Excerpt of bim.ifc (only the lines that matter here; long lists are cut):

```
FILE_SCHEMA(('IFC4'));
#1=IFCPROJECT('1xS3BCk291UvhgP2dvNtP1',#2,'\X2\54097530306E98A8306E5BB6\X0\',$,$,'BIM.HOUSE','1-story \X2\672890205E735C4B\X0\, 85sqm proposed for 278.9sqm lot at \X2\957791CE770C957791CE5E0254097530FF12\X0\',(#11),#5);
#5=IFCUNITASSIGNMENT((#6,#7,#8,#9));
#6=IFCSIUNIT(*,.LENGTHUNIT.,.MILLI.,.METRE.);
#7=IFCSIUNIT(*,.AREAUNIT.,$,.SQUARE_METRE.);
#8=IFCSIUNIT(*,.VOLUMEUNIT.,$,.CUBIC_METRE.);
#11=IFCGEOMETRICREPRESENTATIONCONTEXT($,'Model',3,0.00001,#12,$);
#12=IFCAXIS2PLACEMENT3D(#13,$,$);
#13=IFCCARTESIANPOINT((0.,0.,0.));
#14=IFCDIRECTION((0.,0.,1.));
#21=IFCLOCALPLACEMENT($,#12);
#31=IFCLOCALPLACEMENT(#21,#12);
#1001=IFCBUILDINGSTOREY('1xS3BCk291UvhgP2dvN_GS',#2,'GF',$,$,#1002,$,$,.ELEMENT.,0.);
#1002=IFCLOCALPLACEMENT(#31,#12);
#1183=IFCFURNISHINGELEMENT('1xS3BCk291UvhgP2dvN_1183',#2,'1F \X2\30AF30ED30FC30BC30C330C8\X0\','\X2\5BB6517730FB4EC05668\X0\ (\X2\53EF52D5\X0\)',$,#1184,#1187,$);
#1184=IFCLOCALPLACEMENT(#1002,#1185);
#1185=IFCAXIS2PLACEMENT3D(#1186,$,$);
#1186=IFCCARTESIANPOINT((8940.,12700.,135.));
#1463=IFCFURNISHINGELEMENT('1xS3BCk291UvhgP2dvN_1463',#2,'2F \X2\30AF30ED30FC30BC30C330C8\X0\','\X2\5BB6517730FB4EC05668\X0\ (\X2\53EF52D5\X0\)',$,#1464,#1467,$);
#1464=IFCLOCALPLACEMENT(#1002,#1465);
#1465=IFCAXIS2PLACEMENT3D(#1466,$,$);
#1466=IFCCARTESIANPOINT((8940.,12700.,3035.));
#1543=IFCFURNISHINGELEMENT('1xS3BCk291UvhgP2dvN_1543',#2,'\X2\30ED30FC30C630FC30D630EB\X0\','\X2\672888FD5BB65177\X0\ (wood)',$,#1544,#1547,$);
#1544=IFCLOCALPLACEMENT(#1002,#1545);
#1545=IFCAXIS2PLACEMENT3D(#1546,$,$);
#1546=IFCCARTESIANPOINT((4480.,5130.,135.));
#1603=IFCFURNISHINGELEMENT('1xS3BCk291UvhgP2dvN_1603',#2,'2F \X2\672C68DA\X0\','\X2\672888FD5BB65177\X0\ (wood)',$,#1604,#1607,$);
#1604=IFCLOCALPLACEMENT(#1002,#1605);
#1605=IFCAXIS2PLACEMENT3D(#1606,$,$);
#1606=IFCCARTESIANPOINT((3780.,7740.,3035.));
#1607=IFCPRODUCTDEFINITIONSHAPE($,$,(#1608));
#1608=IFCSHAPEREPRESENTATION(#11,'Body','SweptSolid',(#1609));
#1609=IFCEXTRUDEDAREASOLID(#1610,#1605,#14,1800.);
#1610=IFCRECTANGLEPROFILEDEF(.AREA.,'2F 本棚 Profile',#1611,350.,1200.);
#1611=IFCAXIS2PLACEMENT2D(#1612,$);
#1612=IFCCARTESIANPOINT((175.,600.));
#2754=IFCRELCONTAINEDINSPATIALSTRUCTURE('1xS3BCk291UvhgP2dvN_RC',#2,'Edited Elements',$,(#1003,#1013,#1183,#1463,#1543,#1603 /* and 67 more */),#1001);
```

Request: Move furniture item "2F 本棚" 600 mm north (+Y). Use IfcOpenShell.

```python
import ifcopenshell
import ifcopenshell.api.geometry
import ifcopenshell.util.placement
import ifcopenshell.util.unit

model = ifcopenshell.open("bim.ifc")
unit_scale = ifcopenshell.util.unit.calculate_unit_scale(model)

item = model.by_guid("1xS3BCk291UvhgP2dvN_1603")
matrix = ifcopenshell.util.placement.get_local_placement(item.ObjectPlacement)
matrix[1, 3] += 0.6 / unit_scale
ifcopenshell.api.geometry.edit_object_placement(model, product=item, matrix=matrix, is_si=False)

print(ifcopenshell.util.placement.get_local_placement(item.ObjectPlacement).round(3) + 0.0)

model.write("bim_edited.ifc")
```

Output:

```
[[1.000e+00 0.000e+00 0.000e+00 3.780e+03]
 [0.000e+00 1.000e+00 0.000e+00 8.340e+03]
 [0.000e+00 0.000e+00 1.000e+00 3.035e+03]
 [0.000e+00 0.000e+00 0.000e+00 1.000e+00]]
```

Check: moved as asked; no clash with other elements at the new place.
